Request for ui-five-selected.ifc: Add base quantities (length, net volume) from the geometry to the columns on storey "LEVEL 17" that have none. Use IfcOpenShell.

First a look at what the model holds.

```python
import ifcopenshell
import ifcopenshell.util.element
import ifcopenshell.util.unit

model = ifcopenshell.open("ui-five-selected.ifc")
print(model.schema)
for unit_type in ("LENGTHUNIT", "AREAUNIT", "VOLUMEUNIT"):
    print(unit_type, ifcopenshell.util.unit.calculate_unit_scale(model, unit_type))
storey = next(s for s in model.by_type("IfcBuildingStorey") if s.Name == "LEVEL 17")
columns = [e for e in ifcopenshell.util.element.get_decomposition(storey) if e.is_a("IfcColumn")]
for e in sorted(columns, key=lambda e: e.id()):
    print(e.id(), e.is_a(), e.Name, list(ifcopenshell.util.element.get_psets(e, qtos_only=True)), sep=" | ")
```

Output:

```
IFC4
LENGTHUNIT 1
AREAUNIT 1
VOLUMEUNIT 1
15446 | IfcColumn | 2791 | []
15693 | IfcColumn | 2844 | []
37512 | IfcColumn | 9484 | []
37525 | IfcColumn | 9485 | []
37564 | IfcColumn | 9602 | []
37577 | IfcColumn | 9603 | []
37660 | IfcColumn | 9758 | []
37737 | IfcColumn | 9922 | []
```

```python
import ifcopenshell
import ifcopenshell.api.pset
import ifcopenshell.geom
import ifcopenshell.util.element
import ifcopenshell.util.shape
import ifcopenshell.util.unit

model = ifcopenshell.open("ui-five-selected.ifc")
unit_scale = ifcopenshell.util.unit.calculate_unit_scale(model)
volume_scale = ifcopenshell.util.unit.calculate_unit_scale(model, "VOLUMEUNIT")
settings = ifcopenshell.geom.settings()

storey = next(s for s in model.by_type("IfcBuildingStorey") if s.Name == "LEVEL 17")
columns = [e for e in ifcopenshell.util.element.get_decomposition(storey) if e.is_a("IfcColumn")]

for e in sorted(columns, key=lambda e: e.id()):
    if ifcopenshell.util.element.get_psets(e, qtos_only=True, should_inherit=False):
        continue
    # Geometry comes back in metres, in the element's own axes.
    shape = ifcopenshell.geom.create_shape(settings, e)
    values = {
        "Length": ifcopenshell.util.shape.get_z(shape.geometry) / unit_scale,
        "NetVolume": ifcopenshell.util.shape.get_volume(shape.geometry) / volume_scale,
    }
    qto = ifcopenshell.api.pset.add_qto(model, product=e, name="Qto_ColumnBaseQuantities")
    ifcopenshell.api.pset.edit_qto(model, qto=qto, properties=values)
    print(e.id(), {k: round(v, 3) for k, v in values.items()})

model.write("ui-five-selected_updated.ifc")
```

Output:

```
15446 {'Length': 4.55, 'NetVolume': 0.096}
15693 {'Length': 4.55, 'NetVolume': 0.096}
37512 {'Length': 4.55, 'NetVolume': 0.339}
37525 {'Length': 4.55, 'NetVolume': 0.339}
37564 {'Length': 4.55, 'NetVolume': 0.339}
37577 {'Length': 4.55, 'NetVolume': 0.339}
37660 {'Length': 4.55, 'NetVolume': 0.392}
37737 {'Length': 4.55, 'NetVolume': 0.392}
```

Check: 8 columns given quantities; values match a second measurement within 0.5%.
